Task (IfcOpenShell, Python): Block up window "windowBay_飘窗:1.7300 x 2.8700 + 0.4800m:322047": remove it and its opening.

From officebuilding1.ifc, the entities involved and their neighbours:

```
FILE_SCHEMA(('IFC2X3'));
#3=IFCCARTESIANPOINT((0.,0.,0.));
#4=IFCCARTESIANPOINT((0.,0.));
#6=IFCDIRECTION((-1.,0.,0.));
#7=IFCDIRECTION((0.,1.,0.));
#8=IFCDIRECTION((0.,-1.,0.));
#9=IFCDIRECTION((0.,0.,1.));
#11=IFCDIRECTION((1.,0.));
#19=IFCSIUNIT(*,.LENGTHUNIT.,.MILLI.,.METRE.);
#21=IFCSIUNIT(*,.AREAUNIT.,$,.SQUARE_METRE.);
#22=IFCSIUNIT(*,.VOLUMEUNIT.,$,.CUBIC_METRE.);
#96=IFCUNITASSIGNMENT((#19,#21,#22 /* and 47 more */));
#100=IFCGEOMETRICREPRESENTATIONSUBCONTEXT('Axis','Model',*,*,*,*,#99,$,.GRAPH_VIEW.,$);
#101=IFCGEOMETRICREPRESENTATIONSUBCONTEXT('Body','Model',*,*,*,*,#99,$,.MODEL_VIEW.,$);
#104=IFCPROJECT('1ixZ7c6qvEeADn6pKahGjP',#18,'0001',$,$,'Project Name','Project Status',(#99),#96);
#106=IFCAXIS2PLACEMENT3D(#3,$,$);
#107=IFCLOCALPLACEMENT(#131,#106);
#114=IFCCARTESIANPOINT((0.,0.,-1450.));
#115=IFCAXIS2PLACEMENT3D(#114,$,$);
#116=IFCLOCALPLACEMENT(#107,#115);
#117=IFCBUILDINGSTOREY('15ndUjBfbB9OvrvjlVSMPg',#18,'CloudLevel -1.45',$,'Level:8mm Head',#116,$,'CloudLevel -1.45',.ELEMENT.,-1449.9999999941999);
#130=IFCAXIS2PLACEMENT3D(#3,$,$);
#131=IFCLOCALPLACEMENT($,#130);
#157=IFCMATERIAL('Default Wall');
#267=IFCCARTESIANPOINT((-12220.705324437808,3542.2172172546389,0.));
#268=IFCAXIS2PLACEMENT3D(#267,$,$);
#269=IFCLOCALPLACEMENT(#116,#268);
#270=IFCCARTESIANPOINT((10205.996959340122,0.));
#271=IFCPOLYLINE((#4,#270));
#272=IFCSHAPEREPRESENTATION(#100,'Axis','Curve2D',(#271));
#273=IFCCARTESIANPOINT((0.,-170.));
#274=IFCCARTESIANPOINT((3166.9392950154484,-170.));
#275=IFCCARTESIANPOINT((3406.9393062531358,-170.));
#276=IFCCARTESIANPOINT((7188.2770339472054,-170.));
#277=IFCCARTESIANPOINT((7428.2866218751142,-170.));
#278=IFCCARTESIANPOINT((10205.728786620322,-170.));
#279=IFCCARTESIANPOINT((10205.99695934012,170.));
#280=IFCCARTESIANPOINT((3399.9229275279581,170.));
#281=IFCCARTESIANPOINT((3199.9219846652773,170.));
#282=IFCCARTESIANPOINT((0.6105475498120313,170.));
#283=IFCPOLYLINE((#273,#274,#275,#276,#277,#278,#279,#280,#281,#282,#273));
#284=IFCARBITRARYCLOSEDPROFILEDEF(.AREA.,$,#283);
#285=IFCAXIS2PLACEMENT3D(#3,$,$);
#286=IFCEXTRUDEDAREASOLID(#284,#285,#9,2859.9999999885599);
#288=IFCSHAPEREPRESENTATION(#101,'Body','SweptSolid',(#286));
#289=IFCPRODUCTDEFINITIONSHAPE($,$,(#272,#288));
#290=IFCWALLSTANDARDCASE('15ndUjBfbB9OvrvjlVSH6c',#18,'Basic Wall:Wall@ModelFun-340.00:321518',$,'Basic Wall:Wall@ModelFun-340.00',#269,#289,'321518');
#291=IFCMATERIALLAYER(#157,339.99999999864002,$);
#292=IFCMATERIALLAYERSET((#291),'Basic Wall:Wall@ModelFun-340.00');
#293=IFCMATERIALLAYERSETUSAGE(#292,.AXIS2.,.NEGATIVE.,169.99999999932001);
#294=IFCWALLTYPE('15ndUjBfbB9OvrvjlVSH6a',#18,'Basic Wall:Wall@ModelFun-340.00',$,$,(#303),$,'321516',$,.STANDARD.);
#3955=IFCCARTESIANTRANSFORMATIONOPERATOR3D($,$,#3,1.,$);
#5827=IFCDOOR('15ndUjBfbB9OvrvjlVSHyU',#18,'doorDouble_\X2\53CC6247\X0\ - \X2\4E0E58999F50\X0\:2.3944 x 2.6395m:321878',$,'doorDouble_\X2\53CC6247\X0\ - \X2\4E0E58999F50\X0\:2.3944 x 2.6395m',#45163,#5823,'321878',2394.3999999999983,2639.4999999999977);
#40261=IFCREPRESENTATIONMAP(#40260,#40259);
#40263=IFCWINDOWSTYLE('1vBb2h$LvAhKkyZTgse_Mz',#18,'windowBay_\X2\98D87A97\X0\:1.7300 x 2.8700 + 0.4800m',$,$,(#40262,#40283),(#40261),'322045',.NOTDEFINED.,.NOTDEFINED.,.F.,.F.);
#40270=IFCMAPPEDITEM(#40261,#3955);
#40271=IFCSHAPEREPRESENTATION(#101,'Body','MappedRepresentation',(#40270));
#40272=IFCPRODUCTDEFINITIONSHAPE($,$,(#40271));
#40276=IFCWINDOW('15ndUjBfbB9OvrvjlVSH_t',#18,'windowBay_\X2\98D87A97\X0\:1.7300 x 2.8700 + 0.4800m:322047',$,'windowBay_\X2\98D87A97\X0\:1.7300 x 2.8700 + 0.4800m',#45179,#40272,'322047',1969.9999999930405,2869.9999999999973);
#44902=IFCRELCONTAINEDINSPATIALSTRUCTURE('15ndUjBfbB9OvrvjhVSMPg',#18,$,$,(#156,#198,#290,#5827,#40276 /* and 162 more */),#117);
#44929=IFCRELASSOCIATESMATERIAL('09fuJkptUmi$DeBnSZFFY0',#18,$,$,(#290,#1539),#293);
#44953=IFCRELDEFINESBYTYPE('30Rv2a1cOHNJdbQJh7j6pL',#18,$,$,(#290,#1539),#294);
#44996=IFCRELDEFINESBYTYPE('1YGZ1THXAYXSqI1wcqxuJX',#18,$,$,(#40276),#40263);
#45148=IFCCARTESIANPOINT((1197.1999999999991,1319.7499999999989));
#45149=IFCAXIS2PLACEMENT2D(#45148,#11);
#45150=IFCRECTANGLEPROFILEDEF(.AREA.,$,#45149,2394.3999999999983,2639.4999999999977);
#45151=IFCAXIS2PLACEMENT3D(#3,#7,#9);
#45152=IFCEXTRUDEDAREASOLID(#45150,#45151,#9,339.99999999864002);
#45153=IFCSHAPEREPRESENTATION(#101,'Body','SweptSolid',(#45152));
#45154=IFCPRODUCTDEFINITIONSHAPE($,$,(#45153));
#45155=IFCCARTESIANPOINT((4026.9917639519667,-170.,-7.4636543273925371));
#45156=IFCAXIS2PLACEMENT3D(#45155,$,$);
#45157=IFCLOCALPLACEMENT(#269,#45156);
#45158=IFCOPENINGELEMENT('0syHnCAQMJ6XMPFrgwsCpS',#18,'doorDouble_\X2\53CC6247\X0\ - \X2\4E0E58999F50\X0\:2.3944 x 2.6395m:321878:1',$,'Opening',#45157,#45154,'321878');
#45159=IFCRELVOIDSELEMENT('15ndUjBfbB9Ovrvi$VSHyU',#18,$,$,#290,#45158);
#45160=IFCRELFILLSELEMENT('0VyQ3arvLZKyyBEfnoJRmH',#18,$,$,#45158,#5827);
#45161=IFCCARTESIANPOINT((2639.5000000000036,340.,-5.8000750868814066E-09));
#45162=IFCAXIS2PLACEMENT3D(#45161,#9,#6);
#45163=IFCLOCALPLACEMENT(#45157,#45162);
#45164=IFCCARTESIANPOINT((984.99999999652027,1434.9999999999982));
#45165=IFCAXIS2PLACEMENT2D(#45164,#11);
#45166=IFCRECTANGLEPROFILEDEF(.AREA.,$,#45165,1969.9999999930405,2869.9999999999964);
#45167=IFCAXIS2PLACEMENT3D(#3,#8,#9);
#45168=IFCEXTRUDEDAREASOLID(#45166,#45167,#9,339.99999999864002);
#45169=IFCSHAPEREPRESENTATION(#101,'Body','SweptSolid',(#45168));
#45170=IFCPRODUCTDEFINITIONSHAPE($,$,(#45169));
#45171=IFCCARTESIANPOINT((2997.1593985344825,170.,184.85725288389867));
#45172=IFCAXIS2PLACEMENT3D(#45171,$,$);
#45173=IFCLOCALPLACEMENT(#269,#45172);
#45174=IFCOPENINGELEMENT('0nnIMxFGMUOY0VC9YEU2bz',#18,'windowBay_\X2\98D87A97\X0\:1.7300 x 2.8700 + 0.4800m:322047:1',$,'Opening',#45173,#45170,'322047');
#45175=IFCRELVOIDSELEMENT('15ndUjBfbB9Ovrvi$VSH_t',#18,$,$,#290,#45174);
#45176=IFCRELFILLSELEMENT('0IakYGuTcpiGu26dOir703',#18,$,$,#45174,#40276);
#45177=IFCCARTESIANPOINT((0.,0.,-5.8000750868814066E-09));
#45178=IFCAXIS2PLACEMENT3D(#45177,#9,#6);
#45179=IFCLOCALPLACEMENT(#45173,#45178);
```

```python
import ifcopenshell
import ifcopenshell.api.feature
import ifcopenshell.api.root
import ifcopenshell.geom
import ifcopenshell.util.shape

model = ifcopenshell.open("officebuilding1.ifc")
settings = ifcopenshell.geom.settings()


def volume(element):
    """Net volume in cubic metres, openings subtracted."""
    shape = ifcopenshell.geom.create_shape(settings, element)
    return ifcopenshell.util.shape.get_volume(shape.geometry)


window = model.by_guid("15ndUjBfbB9OvrvjlVSH_t")
opening = window.FillsVoids[0].RelatingOpeningElement
wall = opening.VoidsElements[0].RelatingBuildingElement
before = volume(wall)

ifcopenshell.api.root.remove_product(model, product=window)
ifcopenshell.api.feature.remove_feature(model, feature=opening)

after = volume(wall)

print(f"wall volume {before:.3f} -> {after:.3f} m3")

model.write("officebuilding1-out.ifc")
```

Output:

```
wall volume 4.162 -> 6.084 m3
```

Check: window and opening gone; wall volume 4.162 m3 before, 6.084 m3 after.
